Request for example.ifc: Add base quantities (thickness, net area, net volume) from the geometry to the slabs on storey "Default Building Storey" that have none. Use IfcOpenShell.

First a look at what the model holds.

```python
import ifcopenshell
import ifcopenshell.util.element
import ifcopenshell.util.unit

model = ifcopenshell.open("example.ifc")
print(model.schema)
for unit_type in ("LENGTHUNIT", "AREAUNIT", "VOLUMEUNIT"):
    print(unit_type, ifcopenshell.util.unit.calculate_unit_scale(model, unit_type))
storey = next(s for s in model.by_type("IfcBuildingStorey") if s.Name == "Default Building Storey")
slabs = [e for e in ifcopenshell.util.element.get_decomposition(storey) if e.is_a("IfcSlab")]
for e in sorted(slabs, key=lambda e: e.id()):
    print(e.id(), e.is_a(), e.Name, list(ifcopenshell.util.element.get_psets(e, qtos_only=True)), sep=" | ")
```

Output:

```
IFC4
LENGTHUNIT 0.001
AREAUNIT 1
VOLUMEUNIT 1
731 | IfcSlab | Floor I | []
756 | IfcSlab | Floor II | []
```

```python
import ifcopenshell
import ifcopenshell.api.pset
import ifcopenshell.geom
import ifcopenshell.util.element
import ifcopenshell.util.shape
import ifcopenshell.util.unit

model = ifcopenshell.open("example.ifc")
unit_scale = ifcopenshell.util.unit.calculate_unit_scale(model)
area_scale = ifcopenshell.util.unit.calculate_unit_scale(model, "AREAUNIT")
volume_scale = ifcopenshell.util.unit.calculate_unit_scale(model, "VOLUMEUNIT")
settings = ifcopenshell.geom.settings()

storey = next(s for s in model.by_type("IfcBuildingStorey") if s.Name == "Default Building Storey")
slabs = [e for e in ifcopenshell.util.element.get_decomposition(storey) if e.is_a("IfcSlab")]

for e in sorted(slabs, key=lambda e: e.id()):
    if ifcopenshell.util.element.get_psets(e, qtos_only=True, should_inherit=False):
        continue
    # Geometry comes back in metres, in the element's own axes.
    shape = ifcopenshell.geom.create_shape(settings, e)
    values = {
        "Width": ifcopenshell.util.shape.get_z(shape.geometry) / unit_scale,
        "NetArea": ifcopenshell.util.shape.get_footprint_area(shape.geometry) / area_scale,
        "NetVolume": ifcopenshell.util.shape.get_volume(shape.geometry) / volume_scale,
    }
    qto = ifcopenshell.api.pset.add_qto(model, product=e, name="Qto_SlabBaseQuantities")
    ifcopenshell.api.pset.edit_qto(model, qto=qto, properties=values)
    print(e.id(), {k: round(v, 3) for k, v in values.items()})

model.write("example_rev.ifc")
```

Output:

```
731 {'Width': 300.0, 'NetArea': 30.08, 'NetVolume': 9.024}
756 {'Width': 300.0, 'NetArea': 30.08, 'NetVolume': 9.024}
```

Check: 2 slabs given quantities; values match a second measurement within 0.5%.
